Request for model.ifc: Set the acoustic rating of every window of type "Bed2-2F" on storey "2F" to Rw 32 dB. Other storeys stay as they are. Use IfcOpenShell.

First a look at what the model holds.

```python
import ifcopenshell
import ifcopenshell.util.element

model = ifcopenshell.open("model.ifc")
print(model.schema)
storey = next(s for s in model.by_type("IfcBuildingStorey") if s.Name == "2F")
windows = [e for e in ifcopenshell.util.element.get_decomposition(storey) if e.is_a("IfcWindow")]
seen = {}
for e in windows:
    element_type = ifcopenshell.util.element.get_type(e)
    key = (element_type.Name if element_type != e and element_type else None, ifcopenshell.util.element.get_pset(e, "Pset_WindowCommon", "AcousticRating"))
    seen[key] = seen.get(key, 0) + 1
for (name, value), count in sorted(seen.items(), key=str):
    print(count, "x", name, "|", value)
```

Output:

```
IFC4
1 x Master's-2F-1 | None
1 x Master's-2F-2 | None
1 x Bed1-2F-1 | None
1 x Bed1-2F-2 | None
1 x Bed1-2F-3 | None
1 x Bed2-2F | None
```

```python
import ifcopenshell
import ifcopenshell.api.pset
import ifcopenshell.util.element

model = ifcopenshell.open("model.ifc")

storey = next(s for s in model.by_type("IfcBuildingStorey") if s.Name == "2F")
windows = [e for e in ifcopenshell.util.element.get_decomposition(storey) if e.is_a("IfcWindow")]

count = 0
for e in windows:
    element_type = ifcopenshell.util.element.get_type(e)
    if element_type in (None, e) or element_type.Name != "Bed2-2F":
        continue
    # add_pset returns the element's existing set when there is one.
    pset = ifcopenshell.api.pset.add_pset(model, product=e, name="Pset_WindowCommon")
    ifcopenshell.api.pset.edit_pset(model, pset=pset, properties={"AcousticRating": "Rw 32 dB"})
    count += 1

print(count, "windows updated")

model.write("model_v2.ifc")
```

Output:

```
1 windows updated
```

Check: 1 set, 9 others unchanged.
